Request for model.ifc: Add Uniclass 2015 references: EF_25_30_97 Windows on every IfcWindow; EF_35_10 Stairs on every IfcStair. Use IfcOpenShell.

First a look at what the model holds.

```python
import ifcopenshell

model = ifcopenshell.open("model.ifc")
print(model.schema)
print("classifications:", [c.Name for c in model.by_type("IfcClassification")])
for ifc_class in ("IfcDoor", "IfcRoof", "IfcStair", "IfcWall", "IfcWindow"):
    print(ifc_class, len(model.by_type(ifc_class)))
```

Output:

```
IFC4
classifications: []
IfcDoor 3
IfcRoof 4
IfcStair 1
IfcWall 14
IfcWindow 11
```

```python
import ifcopenshell
import ifcopenshell.api.classification

model = ifcopenshell.open("model.ifc")

system = ifcopenshell.api.classification.add_classification(model, classification="Uniclass 2015")

codes = {
    "IfcWindow": ("EF_25_30_97", "Windows"),
    "IfcStair": ("EF_35_10", "Stairs"),
}
for ifc_class, (code, name) in codes.items():
    products = model.by_type(ifc_class)
    ifcopenshell.api.classification.add_reference(
        model, products=products, classification=system, identification=code, name=name
    )
    print(code, len(products))

model.write("model_updated.ifc")
```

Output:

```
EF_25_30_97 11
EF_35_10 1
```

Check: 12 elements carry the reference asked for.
